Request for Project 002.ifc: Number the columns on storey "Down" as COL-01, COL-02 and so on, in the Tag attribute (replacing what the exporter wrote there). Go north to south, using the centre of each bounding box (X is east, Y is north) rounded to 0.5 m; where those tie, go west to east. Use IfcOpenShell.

First a look at what the model holds.

```python
import ifcopenshell
import ifcopenshell.util.element
import ifcopenshell.util.placement

model = ifcopenshell.open("Project 002.ifc")
print(model.schema)
storey = next(s for s in model.by_type("IfcBuildingStorey") if s.Name == "Down")
columns = [e for e in ifcopenshell.util.element.get_decomposition(storey) if e.is_a("IfcColumn")]
for e in sorted(columns, key=lambda e: e.id()):
    origin = ifcopenshell.util.placement.get_local_placement(e.ObjectPlacement)[:3, 3]
    print(e.id(), e.Tag, e.Name, origin.round(2) + 0.0, sep=" | ")
```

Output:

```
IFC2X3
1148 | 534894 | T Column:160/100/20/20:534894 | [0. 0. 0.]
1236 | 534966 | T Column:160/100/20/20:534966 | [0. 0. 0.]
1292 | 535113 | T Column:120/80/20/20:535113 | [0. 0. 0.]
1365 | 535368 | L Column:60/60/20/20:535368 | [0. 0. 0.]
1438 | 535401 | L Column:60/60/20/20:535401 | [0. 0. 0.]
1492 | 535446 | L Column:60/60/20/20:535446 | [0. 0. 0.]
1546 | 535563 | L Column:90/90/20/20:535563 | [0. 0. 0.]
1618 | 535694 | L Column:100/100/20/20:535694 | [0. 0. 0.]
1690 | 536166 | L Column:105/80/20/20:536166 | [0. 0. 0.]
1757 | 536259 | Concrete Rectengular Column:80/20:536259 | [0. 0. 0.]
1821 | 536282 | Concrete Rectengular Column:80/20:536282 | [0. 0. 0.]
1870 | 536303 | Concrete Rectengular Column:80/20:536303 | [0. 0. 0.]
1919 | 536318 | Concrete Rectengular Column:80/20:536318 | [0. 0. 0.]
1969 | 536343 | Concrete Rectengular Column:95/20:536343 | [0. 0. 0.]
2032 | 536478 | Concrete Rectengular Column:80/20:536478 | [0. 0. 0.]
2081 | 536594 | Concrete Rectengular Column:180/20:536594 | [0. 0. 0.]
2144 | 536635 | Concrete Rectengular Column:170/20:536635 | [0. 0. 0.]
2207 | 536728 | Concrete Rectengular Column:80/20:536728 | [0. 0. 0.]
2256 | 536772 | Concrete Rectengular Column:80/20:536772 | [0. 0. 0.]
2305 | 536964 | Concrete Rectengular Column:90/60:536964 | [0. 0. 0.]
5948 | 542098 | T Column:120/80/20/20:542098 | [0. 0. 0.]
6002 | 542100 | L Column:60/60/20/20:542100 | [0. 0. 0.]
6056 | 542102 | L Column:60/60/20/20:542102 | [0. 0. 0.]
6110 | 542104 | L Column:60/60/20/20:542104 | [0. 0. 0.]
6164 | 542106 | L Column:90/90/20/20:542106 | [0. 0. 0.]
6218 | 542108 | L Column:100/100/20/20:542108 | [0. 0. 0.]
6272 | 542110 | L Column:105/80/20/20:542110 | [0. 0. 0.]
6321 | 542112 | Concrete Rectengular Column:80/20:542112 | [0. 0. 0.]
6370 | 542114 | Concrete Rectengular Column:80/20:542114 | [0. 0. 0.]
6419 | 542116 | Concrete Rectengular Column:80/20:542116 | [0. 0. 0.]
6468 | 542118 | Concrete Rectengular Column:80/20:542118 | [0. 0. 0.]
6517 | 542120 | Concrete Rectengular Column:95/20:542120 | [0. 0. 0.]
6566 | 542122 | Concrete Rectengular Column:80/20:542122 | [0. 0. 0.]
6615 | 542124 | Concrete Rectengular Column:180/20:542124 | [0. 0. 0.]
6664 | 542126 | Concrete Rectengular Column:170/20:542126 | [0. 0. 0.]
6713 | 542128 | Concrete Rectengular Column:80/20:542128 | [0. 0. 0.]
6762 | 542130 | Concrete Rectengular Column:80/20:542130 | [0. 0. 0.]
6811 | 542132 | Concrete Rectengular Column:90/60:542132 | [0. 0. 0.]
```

```python
import ifcopenshell
import ifcopenshell.geom
import ifcopenshell.util.element
import ifcopenshell.util.shape

model = ifcopenshell.open("Project 002.ifc")
settings = ifcopenshell.geom.settings()
settings.set("use-world-coords", True)


def centre(element):
    shape = ifcopenshell.geom.create_shape(settings, element)
    return ifcopenshell.util.shape.get_bbox_centroid(shape.geometry)


storey = next(s for s in model.by_type("IfcBuildingStorey") if s.Name == "Down")
columns = [e for e in ifcopenshell.util.element.get_decomposition(storey) if e.is_a("IfcColumn")]

# Insertion points can sit at a corner or the storey origin, so sort by the geometry (in metres).
centres = {e: centre(e) for e in columns}
columns.sort(key=lambda e: (-round(centres[e][1] / 0.5), centres[e][0]))

for i, e in enumerate(columns, start=1):
    number = f"COL-{i:02d}"
    e.Tag = number
    print(e.id(), number)

model.write("Project 002_edited.ifc")
```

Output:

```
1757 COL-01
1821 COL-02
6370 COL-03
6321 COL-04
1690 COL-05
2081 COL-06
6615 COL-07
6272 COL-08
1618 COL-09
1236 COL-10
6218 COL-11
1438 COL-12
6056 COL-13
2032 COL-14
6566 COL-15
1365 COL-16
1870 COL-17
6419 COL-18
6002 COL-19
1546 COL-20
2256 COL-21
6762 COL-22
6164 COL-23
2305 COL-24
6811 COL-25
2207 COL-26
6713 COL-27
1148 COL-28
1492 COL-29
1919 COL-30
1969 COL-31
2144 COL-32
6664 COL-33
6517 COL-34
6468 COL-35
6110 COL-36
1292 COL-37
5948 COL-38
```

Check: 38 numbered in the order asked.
